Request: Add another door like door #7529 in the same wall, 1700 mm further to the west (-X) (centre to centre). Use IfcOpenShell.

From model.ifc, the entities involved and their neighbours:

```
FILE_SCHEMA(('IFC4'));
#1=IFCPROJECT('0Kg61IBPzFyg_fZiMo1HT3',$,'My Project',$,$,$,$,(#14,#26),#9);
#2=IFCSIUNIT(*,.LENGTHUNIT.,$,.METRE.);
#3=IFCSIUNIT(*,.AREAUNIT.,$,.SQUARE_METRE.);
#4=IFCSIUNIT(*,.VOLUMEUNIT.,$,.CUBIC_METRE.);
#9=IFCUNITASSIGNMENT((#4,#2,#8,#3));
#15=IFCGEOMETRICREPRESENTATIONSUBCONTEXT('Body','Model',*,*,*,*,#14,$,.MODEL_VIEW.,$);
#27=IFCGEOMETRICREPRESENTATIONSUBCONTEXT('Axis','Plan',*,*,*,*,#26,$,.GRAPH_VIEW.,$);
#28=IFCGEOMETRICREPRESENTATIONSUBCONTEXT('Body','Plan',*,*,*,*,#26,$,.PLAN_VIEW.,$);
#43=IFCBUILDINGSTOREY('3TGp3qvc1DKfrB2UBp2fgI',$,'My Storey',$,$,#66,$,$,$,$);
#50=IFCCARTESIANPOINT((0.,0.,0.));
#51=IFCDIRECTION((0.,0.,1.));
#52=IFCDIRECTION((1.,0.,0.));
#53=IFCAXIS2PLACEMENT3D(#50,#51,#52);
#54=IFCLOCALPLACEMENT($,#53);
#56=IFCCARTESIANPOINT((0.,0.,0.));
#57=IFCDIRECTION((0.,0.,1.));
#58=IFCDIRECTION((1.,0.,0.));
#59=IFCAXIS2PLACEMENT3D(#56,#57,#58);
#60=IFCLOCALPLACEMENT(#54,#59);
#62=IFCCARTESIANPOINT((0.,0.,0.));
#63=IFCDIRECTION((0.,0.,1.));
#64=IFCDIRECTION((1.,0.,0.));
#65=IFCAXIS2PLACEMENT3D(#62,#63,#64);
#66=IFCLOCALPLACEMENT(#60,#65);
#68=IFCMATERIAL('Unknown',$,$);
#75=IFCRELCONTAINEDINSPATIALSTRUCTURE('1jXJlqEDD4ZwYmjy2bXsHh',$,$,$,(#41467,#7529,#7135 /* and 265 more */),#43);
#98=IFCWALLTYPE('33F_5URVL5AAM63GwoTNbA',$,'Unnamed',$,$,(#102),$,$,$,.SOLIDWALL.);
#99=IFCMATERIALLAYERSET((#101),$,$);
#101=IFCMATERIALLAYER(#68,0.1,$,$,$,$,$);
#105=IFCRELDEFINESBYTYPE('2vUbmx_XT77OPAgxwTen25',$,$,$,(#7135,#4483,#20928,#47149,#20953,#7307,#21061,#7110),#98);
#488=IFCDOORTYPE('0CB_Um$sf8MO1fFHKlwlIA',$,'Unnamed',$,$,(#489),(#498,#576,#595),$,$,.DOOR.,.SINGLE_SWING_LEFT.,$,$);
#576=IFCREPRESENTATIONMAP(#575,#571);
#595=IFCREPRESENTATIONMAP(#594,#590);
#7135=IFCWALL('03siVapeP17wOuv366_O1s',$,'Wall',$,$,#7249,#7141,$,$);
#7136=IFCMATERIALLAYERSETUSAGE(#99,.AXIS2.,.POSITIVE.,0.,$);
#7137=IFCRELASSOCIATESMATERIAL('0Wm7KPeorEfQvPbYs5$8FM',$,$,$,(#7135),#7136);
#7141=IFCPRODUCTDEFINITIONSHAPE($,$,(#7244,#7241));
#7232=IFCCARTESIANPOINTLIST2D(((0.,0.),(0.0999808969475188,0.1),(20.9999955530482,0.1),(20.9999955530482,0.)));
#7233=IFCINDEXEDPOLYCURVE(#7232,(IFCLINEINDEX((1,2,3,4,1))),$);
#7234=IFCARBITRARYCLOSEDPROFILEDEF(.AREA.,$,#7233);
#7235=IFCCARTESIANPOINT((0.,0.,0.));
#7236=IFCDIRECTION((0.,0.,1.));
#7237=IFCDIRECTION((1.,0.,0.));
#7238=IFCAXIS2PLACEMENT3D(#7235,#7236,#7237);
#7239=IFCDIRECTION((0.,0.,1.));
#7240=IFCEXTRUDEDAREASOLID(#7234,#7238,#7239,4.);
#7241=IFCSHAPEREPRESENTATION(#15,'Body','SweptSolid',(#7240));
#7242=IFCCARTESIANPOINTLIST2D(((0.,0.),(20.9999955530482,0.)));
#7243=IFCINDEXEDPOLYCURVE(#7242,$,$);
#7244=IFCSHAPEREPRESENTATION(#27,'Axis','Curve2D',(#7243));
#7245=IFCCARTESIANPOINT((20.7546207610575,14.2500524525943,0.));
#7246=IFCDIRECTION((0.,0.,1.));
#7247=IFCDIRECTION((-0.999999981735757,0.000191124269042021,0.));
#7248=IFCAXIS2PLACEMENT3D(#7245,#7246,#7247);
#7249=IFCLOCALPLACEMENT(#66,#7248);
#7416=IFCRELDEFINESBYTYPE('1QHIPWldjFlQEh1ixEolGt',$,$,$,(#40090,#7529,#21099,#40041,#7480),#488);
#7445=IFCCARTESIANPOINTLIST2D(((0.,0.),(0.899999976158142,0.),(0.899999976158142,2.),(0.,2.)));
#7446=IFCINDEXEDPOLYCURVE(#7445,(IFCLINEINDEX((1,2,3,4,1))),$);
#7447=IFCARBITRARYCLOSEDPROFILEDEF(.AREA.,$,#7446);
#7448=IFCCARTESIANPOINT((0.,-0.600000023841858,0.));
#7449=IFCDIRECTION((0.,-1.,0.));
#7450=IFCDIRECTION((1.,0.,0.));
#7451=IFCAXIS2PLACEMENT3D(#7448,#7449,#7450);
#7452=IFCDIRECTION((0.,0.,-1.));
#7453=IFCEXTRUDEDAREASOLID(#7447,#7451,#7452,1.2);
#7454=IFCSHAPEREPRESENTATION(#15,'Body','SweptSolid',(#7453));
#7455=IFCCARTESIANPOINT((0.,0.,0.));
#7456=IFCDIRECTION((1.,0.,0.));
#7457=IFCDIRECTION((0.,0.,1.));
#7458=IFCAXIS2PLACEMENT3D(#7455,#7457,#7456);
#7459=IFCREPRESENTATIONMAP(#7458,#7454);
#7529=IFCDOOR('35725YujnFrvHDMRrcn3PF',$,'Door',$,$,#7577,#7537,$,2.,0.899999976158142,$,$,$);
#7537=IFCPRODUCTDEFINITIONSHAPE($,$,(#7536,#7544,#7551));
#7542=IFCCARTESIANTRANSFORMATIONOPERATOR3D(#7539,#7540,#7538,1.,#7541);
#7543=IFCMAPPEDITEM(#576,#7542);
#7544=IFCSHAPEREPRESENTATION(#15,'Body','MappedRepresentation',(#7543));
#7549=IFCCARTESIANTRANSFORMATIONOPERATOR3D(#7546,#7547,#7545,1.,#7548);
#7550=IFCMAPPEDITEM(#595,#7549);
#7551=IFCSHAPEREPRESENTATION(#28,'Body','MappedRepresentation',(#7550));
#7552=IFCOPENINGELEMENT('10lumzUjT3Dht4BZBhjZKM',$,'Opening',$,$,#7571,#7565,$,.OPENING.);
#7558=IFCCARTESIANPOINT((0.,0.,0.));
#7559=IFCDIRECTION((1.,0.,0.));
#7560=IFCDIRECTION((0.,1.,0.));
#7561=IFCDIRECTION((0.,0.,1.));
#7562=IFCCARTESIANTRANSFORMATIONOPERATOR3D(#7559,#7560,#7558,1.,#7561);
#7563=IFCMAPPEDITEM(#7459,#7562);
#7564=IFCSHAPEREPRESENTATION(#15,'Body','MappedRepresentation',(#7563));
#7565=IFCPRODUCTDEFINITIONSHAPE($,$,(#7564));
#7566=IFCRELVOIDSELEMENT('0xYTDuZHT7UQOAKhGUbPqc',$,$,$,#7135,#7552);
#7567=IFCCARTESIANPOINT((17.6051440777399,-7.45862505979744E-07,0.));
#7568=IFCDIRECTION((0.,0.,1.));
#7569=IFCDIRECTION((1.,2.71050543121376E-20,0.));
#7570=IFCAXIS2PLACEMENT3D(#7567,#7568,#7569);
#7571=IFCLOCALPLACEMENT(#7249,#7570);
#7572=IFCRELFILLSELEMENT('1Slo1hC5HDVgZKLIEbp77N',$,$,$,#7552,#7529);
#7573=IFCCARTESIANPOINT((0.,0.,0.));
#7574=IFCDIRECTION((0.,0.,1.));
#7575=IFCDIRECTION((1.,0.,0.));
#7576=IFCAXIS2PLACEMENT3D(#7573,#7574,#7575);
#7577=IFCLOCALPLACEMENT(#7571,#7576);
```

```python
import ifcopenshell
import ifcopenshell.api.feature
import ifcopenshell.api.geometry
import ifcopenshell.api.root
import ifcopenshell.geom
import ifcopenshell.util.element
import ifcopenshell.util.placement
import ifcopenshell.util.shape
import ifcopenshell.util.unit

model = ifcopenshell.open("model.ifc")
unit_scale = ifcopenshell.util.unit.calculate_unit_scale(model)
settings = ifcopenshell.geom.settings()


def volume(element):
    """Net volume in cubic metres, openings subtracted."""
    shape = ifcopenshell.geom.create_shape(settings, element)
    return ifcopenshell.util.shape.get_volume(shape.geometry)


door = model.by_id(7529)
opening = door.FillsVoids[0].RelatingOpeningElement
wall = opening.VoidsElements[0].RelatingBuildingElement
before = volume(wall)
shift = ifcopenshell.util.placement.get_local_placement(wall.ObjectPlacement)[:3, 0] * 1.7 / unit_scale

# copy_class copies the void relationship, type, container and properties, but no geometry.
new_opening = ifcopenshell.api.root.copy_class(model, product=opening)
new_opening.Representation = ifcopenshell.util.element.copy_deep(
    model, opening.Representation, exclude=["IfcGeometricRepresentationContext", "IfcRepresentationMap"]
)
new_door = ifcopenshell.api.root.copy_class(model, product=door)
new_door.Representation = ifcopenshell.util.element.copy_deep(
    model, door.Representation, exclude=["IfcGeometricRepresentationContext", "IfcRepresentationMap"]
)
ifcopenshell.api.feature.add_filling(model, opening=new_opening, element=new_door)

for old, new in ((opening, new_opening), (door, new_door)):
    matrix = ifcopenshell.util.placement.get_local_placement(old.ObjectPlacement)
    matrix[:3, 3] += shift
    ifcopenshell.api.geometry.edit_object_placement(model, product=new, matrix=matrix, is_si=False)

after = volume(wall)

print(f"wall volume {before:.3f} -> {after:.3f} m3")

model.write("model_updated.ifc")
```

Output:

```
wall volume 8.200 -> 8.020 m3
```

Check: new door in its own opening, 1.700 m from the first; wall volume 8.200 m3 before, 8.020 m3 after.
